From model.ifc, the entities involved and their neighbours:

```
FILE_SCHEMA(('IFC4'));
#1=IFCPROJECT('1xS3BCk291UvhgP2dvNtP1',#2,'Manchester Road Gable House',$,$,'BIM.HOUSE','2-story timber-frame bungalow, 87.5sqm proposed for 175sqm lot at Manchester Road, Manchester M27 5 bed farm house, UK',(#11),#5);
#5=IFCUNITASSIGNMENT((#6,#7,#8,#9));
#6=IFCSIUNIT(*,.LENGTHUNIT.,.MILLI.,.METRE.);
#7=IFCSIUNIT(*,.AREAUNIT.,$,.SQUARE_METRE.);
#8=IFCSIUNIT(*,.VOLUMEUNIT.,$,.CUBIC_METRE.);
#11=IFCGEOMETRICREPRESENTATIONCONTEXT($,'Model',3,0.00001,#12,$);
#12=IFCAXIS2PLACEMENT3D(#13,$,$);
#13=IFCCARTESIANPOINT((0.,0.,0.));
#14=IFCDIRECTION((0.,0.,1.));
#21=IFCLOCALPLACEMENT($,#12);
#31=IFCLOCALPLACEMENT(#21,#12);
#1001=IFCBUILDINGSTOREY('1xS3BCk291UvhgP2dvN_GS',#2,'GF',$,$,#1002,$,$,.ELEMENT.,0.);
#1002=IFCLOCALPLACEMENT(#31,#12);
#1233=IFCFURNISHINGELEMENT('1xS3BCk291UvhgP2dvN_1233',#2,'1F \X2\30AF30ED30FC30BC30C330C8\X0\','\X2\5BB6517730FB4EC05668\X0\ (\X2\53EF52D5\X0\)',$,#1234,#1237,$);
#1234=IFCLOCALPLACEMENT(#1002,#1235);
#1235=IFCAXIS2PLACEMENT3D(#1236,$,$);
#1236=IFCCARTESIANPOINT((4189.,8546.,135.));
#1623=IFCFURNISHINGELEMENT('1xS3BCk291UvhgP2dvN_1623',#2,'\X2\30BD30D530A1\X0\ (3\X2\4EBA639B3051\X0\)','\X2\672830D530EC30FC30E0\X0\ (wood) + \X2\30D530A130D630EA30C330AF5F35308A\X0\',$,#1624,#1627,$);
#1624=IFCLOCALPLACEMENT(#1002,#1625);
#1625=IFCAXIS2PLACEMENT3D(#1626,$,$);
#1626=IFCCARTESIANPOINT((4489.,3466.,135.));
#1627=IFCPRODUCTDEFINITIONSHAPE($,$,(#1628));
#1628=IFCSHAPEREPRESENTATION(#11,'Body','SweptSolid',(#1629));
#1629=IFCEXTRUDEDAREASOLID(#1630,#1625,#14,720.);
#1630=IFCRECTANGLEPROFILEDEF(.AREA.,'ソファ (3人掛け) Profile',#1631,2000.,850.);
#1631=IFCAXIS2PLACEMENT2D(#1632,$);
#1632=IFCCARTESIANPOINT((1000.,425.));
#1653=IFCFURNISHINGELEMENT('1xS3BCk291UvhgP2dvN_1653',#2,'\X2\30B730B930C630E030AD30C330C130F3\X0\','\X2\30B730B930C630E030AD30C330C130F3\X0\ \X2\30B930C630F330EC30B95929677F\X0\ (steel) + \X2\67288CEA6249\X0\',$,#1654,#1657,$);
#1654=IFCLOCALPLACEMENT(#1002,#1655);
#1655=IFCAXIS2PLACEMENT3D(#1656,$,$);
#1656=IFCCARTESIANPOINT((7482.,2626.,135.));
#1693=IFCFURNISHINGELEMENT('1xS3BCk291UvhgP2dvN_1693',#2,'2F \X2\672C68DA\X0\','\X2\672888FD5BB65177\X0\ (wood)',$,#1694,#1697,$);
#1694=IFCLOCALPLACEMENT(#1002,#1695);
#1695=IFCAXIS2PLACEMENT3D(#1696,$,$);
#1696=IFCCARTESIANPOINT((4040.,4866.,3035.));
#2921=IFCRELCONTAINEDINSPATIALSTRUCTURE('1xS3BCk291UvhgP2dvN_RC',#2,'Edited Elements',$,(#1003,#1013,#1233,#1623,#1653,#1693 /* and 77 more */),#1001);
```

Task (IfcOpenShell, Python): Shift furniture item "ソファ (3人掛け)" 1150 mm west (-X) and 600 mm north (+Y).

```python
import ifcopenshell
import ifcopenshell.api.geometry
import ifcopenshell.util.placement
import ifcopenshell.util.unit

model = ifcopenshell.open("model.ifc")
unit_scale = ifcopenshell.util.unit.calculate_unit_scale(model)

item = model.by_guid("1xS3BCk291UvhgP2dvN_1623")
matrix = ifcopenshell.util.placement.get_local_placement(item.ObjectPlacement)
matrix[0, 3] -= 1.15 / unit_scale
matrix[1, 3] += 0.6 / unit_scale
ifcopenshell.api.geometry.edit_object_placement(model, product=item, matrix=matrix, is_si=False)

print(ifcopenshell.util.placement.get_local_placement(item.ObjectPlacement).round(3) + 0.0)

model.write("model_edited.ifc")
```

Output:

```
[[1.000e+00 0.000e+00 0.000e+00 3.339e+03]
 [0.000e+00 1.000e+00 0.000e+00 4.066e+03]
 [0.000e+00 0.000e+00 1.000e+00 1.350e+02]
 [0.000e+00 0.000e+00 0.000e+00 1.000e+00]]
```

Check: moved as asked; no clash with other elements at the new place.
